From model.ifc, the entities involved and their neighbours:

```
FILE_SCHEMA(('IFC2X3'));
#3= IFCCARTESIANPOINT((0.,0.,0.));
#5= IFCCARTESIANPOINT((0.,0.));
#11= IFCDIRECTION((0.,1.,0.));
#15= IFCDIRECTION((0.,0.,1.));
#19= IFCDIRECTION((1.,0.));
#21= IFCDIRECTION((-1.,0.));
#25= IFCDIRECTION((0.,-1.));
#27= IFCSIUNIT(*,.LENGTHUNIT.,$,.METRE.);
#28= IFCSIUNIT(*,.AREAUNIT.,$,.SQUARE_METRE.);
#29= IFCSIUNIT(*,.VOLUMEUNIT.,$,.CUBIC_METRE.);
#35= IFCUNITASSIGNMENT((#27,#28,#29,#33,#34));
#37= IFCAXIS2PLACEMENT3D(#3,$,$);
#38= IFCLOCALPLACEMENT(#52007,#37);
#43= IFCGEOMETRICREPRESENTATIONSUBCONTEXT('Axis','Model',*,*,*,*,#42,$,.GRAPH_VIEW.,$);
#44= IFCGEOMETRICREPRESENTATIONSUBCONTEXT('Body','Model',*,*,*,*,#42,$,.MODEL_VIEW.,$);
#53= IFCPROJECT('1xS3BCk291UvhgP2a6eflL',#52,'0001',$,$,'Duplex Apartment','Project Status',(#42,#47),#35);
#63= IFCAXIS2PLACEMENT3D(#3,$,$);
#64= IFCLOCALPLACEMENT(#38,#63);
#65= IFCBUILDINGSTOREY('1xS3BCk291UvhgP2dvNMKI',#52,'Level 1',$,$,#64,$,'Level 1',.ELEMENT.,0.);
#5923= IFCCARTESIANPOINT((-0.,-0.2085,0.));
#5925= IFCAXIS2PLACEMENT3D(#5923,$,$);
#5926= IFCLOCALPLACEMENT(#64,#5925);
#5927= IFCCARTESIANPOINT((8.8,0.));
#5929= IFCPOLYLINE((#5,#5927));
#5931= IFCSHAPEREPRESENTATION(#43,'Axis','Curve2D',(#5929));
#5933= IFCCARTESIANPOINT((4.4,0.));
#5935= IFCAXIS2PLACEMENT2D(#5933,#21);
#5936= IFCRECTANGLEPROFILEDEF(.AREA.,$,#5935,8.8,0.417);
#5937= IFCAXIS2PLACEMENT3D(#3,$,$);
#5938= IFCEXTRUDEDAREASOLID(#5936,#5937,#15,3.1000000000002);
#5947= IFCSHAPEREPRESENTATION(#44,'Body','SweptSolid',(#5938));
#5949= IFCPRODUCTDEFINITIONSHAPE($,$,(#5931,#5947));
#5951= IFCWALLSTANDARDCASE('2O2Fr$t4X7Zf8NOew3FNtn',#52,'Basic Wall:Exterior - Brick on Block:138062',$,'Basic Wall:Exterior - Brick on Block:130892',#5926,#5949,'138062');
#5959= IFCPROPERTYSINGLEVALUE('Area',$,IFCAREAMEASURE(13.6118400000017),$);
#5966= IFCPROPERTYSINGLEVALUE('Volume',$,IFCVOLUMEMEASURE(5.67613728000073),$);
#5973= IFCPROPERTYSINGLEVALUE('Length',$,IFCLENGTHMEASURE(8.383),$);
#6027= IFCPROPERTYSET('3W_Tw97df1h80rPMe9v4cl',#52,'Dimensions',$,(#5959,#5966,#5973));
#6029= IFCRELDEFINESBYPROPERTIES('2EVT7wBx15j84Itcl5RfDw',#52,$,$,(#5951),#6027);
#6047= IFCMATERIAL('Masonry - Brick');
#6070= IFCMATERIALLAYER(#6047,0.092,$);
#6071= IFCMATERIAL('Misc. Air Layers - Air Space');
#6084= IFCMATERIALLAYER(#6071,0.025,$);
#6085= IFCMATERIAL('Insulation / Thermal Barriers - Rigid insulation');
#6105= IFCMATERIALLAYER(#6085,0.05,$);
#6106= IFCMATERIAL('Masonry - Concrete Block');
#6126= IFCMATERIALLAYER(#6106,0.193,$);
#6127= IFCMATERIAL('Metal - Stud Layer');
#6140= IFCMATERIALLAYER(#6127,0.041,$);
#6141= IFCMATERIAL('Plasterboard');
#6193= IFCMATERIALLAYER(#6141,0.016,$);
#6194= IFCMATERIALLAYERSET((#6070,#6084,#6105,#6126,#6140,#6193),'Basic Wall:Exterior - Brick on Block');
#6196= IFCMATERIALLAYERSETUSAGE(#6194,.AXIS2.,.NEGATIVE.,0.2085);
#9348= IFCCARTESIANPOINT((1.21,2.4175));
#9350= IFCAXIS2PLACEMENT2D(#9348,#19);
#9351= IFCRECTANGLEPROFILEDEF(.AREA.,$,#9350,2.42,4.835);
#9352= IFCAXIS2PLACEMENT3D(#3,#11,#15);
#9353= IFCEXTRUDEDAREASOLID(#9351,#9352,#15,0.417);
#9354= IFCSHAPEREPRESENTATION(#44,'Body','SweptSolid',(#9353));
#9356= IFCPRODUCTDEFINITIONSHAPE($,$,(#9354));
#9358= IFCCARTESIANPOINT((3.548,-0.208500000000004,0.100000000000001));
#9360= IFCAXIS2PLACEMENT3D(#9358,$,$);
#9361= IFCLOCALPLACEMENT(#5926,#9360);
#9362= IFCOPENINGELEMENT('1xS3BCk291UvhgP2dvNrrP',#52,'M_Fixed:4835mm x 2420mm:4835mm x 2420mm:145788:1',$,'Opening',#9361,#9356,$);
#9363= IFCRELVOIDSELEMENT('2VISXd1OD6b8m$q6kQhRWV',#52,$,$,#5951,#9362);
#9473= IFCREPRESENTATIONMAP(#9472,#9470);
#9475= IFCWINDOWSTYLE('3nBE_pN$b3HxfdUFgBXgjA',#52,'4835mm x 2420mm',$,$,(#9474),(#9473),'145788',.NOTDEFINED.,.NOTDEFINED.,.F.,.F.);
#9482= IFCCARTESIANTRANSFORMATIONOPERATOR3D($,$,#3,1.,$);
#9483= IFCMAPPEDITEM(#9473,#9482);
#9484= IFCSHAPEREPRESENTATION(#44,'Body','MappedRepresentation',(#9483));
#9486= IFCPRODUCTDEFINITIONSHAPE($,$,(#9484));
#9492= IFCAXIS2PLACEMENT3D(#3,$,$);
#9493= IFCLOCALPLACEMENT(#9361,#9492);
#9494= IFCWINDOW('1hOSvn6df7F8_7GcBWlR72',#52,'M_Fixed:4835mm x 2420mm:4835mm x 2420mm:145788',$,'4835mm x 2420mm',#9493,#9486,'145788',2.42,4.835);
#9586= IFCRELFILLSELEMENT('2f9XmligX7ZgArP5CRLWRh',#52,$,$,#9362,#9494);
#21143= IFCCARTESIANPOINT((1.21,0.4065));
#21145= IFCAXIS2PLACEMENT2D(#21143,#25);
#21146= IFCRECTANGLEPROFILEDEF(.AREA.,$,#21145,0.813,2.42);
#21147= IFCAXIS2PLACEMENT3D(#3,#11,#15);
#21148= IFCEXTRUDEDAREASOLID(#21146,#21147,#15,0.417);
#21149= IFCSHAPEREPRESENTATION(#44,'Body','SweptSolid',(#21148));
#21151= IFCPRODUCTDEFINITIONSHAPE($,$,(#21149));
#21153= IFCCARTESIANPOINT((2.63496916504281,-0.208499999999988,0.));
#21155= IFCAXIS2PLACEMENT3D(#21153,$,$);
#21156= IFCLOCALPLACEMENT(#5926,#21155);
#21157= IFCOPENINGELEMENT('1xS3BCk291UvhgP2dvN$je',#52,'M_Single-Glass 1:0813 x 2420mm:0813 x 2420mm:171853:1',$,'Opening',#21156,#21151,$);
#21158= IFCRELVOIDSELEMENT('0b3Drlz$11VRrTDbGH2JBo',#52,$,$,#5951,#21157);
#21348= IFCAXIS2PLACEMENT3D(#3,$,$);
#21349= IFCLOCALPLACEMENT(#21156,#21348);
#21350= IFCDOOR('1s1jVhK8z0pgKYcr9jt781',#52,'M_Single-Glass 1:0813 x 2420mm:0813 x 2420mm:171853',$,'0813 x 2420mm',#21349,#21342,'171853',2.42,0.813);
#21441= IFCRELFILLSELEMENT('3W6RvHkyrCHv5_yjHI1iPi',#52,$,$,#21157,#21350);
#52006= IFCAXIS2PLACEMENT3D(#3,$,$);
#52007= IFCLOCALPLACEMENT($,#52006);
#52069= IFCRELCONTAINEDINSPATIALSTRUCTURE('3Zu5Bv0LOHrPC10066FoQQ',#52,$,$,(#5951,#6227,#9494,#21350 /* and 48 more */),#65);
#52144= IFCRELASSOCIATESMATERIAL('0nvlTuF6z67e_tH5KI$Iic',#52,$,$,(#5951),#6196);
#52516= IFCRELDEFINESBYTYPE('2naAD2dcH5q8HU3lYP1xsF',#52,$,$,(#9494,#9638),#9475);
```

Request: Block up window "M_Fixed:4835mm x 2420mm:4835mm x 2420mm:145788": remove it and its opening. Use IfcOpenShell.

```python
import ifcopenshell
import ifcopenshell.api.feature
import ifcopenshell.api.pset
import ifcopenshell.api.root
import ifcopenshell.geom
import ifcopenshell.util.element
import ifcopenshell.util.shape
import ifcopenshell.util.unit

model = ifcopenshell.open("model.ifc")
area_scale = ifcopenshell.util.unit.calculate_unit_scale(model, "AREAUNIT")
volume_scale = ifcopenshell.util.unit.calculate_unit_scale(model, "VOLUMEUNIT")
settings = ifcopenshell.geom.settings()


def volume(element):
    """Net volume in cubic metres, openings subtracted."""
    shape = ifcopenshell.geom.create_shape(settings, element)
    return ifcopenshell.util.shape.get_volume(shape.geometry)


window = model.by_guid("1hOSvn6df7F8_7GcBWlR72")
opening = window.FillsVoids[0].RelatingOpeningElement
wall = opening.VoidsElements[0].RelatingBuildingElement
before = volume(wall)

ifcopenshell.api.root.remove_product(model, product=window)
ifcopenshell.api.feature.remove_feature(model, feature=opening)

after = volume(wall)
thickness = 0.417  # wall thickness in metres

# Update the wall's stored quantities.
pset = model.by_id(ifcopenshell.util.element.get_pset(wall, "Dimensions", should_inherit=False)["id"])
ifcopenshell.api.pset.edit_pset(model, pset=pset, properties={
    "Area": model.create_entity("IfcAreaMeasure", after / thickness / area_scale),
    "Volume": model.create_entity("IfcVolumeMeasure", after / volume_scale),
})

print(f"wall volume {before:.3f} -> {after:.3f} m3")

model.write("model_v2.ifc")
```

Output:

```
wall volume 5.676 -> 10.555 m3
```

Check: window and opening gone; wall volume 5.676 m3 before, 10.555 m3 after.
